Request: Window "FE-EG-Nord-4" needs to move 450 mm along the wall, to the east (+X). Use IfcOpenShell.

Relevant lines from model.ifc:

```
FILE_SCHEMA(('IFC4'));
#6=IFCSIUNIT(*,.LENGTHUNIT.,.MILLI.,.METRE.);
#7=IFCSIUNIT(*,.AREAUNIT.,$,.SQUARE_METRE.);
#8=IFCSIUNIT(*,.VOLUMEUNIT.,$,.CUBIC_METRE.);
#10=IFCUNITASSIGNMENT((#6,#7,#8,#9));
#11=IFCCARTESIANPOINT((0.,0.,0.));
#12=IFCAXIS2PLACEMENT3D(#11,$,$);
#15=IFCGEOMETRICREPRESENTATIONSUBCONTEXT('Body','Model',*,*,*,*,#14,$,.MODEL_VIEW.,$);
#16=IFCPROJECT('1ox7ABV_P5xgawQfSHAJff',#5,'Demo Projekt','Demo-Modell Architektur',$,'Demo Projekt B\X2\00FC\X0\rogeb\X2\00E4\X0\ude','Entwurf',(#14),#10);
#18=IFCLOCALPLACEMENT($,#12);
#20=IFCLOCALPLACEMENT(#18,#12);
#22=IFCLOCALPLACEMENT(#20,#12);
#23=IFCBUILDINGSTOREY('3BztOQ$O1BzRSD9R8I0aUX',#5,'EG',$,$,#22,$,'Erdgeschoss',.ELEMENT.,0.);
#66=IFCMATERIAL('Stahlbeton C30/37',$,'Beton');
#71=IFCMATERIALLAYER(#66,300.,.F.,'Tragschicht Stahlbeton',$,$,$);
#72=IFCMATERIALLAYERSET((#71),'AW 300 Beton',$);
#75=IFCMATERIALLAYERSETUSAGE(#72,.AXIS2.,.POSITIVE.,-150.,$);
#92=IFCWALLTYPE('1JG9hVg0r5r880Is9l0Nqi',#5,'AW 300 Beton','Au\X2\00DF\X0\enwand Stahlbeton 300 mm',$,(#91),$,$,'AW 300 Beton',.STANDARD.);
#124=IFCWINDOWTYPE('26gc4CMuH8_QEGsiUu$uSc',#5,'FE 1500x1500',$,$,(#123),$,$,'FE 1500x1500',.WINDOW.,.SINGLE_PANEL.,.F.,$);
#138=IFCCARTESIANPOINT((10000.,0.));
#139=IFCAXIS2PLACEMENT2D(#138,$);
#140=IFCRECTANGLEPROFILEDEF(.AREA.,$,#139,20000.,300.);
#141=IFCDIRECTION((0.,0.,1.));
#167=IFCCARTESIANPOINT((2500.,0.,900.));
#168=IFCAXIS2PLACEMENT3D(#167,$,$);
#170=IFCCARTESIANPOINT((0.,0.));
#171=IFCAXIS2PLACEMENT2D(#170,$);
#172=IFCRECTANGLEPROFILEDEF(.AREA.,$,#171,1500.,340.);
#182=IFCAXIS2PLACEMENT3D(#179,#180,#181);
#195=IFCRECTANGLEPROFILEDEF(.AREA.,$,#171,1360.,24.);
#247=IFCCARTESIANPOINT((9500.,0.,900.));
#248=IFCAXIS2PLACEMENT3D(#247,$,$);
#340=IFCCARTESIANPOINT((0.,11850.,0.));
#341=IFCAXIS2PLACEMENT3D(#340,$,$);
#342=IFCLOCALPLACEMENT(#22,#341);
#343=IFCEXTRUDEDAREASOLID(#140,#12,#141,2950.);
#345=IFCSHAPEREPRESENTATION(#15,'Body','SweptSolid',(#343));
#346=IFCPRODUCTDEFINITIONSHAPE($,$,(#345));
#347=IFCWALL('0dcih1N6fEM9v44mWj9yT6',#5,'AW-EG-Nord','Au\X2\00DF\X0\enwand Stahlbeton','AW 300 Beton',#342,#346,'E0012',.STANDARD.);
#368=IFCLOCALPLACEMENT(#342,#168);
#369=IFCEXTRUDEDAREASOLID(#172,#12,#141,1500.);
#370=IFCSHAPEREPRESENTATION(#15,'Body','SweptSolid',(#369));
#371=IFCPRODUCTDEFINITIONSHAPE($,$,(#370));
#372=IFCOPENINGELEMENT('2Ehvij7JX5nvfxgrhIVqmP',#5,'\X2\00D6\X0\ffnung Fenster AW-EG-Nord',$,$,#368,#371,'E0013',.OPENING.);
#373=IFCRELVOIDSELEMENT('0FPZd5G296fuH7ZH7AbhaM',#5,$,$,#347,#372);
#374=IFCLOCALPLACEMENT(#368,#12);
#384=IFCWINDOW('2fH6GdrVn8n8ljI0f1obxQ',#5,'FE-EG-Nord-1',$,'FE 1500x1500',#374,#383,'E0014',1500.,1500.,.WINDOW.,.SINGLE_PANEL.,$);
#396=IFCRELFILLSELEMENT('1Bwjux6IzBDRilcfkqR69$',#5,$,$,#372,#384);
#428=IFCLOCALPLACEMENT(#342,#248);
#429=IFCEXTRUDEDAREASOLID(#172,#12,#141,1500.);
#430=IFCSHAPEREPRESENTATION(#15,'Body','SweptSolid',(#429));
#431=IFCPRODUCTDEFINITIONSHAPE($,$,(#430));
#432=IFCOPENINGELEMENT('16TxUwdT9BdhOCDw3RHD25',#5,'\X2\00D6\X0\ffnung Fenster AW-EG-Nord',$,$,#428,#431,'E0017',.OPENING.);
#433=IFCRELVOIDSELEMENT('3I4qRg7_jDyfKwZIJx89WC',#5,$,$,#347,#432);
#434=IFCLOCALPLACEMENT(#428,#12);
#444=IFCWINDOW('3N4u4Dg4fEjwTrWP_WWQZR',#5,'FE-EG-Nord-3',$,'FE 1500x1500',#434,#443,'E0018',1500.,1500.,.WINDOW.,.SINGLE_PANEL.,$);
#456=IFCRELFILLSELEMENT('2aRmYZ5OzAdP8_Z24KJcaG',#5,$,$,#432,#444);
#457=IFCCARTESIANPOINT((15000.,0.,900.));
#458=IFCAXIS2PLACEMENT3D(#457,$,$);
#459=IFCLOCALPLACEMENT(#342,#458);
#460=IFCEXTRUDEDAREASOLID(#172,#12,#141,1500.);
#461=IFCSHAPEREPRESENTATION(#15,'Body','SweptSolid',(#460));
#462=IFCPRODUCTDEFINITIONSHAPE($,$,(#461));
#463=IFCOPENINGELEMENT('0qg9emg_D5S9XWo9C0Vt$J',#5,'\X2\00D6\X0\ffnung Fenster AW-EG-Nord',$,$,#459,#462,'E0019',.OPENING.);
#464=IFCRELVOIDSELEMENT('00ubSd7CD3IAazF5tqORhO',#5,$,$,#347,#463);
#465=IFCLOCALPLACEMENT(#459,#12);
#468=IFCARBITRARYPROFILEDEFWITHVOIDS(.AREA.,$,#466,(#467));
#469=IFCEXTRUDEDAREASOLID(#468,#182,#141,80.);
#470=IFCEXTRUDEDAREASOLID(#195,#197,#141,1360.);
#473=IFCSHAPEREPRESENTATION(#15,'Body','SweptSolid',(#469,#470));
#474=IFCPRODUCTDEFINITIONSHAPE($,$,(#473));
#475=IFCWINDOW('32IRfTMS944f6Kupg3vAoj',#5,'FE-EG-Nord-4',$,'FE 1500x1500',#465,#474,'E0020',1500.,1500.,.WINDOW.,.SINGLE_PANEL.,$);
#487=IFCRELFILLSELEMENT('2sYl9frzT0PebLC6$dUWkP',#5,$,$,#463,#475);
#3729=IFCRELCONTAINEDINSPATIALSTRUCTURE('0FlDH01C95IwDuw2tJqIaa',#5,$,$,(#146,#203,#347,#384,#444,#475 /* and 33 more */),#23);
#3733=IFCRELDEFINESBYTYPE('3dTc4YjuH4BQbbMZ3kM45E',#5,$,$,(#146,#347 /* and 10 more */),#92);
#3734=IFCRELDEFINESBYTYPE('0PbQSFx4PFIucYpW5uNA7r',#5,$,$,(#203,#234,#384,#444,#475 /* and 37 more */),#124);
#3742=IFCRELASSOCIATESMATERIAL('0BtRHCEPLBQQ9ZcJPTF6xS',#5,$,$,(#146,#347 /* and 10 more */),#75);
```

```python
import ifcopenshell
import ifcopenshell.api.geometry
import ifcopenshell.util.placement

model = ifcopenshell.open("model.ifc")

window = model.by_guid("32IRfTMS944f6Kupg3vAoj")
opening = window.FillsVoids[0].RelatingOpeningElement
wall = opening.VoidsElements[0].RelatingBuildingElement

wall_matrix = ifcopenshell.util.placement.get_local_placement(wall.ObjectPlacement)
shift = wall_matrix[:3, 0] * 450.0
before = ifcopenshell.util.placement.get_local_placement(window.ObjectPlacement)[:3, 3].copy()

# The window is placed relative to its opening, so it follows when the opening moves.
matrix = ifcopenshell.util.placement.get_local_placement(opening.ObjectPlacement)
matrix[:3, 3] += shift
ifcopenshell.api.geometry.edit_object_placement(
    model, product=opening, matrix=matrix, is_si=False, should_transform_children=True
)

after = ifcopenshell.util.placement.get_local_placement(window.ObjectPlacement)[:3, 3]
print("window moved by", (after - before).round(3) + 0.0)

model.write("model_rev.ifc")
```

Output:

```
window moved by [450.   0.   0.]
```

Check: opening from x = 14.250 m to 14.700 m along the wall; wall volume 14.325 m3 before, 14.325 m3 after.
